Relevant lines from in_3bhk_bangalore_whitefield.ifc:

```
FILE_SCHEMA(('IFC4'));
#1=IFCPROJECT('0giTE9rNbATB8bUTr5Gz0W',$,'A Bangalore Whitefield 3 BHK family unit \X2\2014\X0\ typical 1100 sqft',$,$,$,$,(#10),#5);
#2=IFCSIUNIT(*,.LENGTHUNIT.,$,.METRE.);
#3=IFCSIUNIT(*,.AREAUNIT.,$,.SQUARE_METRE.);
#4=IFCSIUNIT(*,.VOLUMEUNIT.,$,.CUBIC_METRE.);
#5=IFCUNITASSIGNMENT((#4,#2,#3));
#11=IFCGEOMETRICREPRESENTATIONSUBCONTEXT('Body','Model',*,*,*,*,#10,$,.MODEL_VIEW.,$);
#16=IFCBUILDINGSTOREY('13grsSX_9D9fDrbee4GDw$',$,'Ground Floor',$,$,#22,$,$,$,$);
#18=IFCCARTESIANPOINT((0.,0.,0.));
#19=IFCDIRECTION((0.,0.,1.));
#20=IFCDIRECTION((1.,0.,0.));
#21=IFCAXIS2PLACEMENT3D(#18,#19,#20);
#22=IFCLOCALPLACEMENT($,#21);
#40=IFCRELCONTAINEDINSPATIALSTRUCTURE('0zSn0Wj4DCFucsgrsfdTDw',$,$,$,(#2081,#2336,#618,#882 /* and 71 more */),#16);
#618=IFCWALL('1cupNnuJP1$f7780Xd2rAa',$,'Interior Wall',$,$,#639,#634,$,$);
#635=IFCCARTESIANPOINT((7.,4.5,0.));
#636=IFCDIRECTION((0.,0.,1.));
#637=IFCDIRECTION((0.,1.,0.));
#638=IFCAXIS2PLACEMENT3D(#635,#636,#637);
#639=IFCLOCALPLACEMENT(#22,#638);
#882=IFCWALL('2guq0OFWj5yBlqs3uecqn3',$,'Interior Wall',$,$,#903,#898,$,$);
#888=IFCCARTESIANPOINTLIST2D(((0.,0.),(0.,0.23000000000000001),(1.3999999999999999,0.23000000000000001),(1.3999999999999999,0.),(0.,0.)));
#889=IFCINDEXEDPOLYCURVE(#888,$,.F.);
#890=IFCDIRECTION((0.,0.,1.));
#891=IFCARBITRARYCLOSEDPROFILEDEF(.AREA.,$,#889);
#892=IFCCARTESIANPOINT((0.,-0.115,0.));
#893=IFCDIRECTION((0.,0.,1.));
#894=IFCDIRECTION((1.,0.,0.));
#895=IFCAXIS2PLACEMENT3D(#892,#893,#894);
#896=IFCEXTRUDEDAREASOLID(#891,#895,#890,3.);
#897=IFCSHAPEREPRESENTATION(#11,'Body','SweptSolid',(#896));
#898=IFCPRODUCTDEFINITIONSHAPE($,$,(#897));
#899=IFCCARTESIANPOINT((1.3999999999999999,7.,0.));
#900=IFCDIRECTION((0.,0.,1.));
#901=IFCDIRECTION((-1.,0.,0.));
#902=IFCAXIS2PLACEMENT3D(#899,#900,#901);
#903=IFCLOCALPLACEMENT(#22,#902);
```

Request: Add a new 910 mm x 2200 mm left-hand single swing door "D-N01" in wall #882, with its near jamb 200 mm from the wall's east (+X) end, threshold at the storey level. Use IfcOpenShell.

```python
import numpy as np
import ifcopenshell
import ifcopenshell.api.feature
import ifcopenshell.api.geometry
import ifcopenshell.api.root
import ifcopenshell.api.spatial
import ifcopenshell.geom
import ifcopenshell.util.element
import ifcopenshell.util.placement
import ifcopenshell.util.representation
import ifcopenshell.util.shape
import ifcopenshell.util.unit

model = ifcopenshell.open("in_3bhk_bangalore_whitefield.ifc")
unit_scale = ifcopenshell.util.unit.calculate_unit_scale(model)
settings = ifcopenshell.geom.settings()


def volume(element):
    """Net volume in cubic metres, openings subtracted."""
    shape = ifcopenshell.geom.create_shape(settings, element)
    return ifcopenshell.util.shape.get_volume(shape.geometry)


wall = model.by_guid("2guq0OFWj5yBlqs3uecqn3")
storey = ifcopenshell.util.element.get_container(wall, ifc_class="IfcBuildingStorey")
context = ifcopenshell.util.representation.get_context(model, "Model", "Body", "MODEL_VIEW")
before = volume(wall)

width, height, from_end, sill = 0.91, 2.2, 0.2, 0.0  # metres

# The wall runs along its own X axis, and the end named is its -X end.
wall_shape = ifcopenshell.geom.create_shape(settings, wall)
x, y, z = ifcopenshell.util.shape.get_vertices(wall_shape.geometry).T
start = x.min() + from_end
face, thickness = float(y.min()), float(y.max() - y.min())
wall_matrix = ifcopenshell.util.placement.get_local_placement(wall.ObjectPlacement)
level = ifcopenshell.util.placement.get_local_placement(storey.ObjectPlacement)[2, 3]


def in_wall(x, y):
    """Placement at x, y metres in the wall's axes, at sill height."""
    matrix = wall_matrix.copy()
    matrix[:, 3] = wall_matrix @ np.array([x / unit_scale, y / unit_scale, 0.0, 1.0])
    matrix[2, 3] = level + sill / unit_scale
    return matrix


# Opening: a box that overshoots both wall faces by 50 mm.
opening = ifcopenshell.api.root.create_entity(model, ifc_class="IfcOpeningElement", predefined_type="OPENING")
box = ifcopenshell.api.geometry.add_wall_representation(
    model, context=context, length=width, height=height, thickness=thickness + 0.1
)
ifcopenshell.api.geometry.assign_representation(model, product=opening, representation=box)
ifcopenshell.api.geometry.edit_object_placement(model, product=opening, matrix=in_wall(start, face - 0.05), is_si=False)
ifcopenshell.api.feature.add_feature(model, feature=opening, element=wall)

door = ifcopenshell.api.root.create_entity(model, ifc_class="IfcDoor", name="D-N01", predefined_type="DOOR")
door.OverallWidth, door.OverallHeight = width / unit_scale, height / unit_scale
door.OperationType = "SINGLE_SWING_LEFT"
body = ifcopenshell.api.geometry.add_door_representation(
    model,
    context=context,
    overall_width=door.OverallWidth,
    overall_height=door.OverallHeight,
    operation_type="SINGLE_SWING_LEFT",
    lining_properties={"LiningDepth": thickness / unit_scale, "ThresholdDepth": thickness / unit_scale},
)
ifcopenshell.api.geometry.assign_representation(model, product=door, representation=body)
ifcopenshell.api.spatial.assign_container(model, products=[door], relating_structure=storey)
ifcopenshell.api.feature.add_filling(model, opening=opening, element=door)

# The lining spans the wall, so the door starts at the wall face.
ifcopenshell.api.geometry.edit_object_placement(model, product=door, matrix=in_wall(start, face), is_si=False)

after = volume(wall)

print(f"wall volume {before:.3f} -> {after:.3f} m3")

model.write("in_3bhk_bangalore_whitefield-out.ifc")
```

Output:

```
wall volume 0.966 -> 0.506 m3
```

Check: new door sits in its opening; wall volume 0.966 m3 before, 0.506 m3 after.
